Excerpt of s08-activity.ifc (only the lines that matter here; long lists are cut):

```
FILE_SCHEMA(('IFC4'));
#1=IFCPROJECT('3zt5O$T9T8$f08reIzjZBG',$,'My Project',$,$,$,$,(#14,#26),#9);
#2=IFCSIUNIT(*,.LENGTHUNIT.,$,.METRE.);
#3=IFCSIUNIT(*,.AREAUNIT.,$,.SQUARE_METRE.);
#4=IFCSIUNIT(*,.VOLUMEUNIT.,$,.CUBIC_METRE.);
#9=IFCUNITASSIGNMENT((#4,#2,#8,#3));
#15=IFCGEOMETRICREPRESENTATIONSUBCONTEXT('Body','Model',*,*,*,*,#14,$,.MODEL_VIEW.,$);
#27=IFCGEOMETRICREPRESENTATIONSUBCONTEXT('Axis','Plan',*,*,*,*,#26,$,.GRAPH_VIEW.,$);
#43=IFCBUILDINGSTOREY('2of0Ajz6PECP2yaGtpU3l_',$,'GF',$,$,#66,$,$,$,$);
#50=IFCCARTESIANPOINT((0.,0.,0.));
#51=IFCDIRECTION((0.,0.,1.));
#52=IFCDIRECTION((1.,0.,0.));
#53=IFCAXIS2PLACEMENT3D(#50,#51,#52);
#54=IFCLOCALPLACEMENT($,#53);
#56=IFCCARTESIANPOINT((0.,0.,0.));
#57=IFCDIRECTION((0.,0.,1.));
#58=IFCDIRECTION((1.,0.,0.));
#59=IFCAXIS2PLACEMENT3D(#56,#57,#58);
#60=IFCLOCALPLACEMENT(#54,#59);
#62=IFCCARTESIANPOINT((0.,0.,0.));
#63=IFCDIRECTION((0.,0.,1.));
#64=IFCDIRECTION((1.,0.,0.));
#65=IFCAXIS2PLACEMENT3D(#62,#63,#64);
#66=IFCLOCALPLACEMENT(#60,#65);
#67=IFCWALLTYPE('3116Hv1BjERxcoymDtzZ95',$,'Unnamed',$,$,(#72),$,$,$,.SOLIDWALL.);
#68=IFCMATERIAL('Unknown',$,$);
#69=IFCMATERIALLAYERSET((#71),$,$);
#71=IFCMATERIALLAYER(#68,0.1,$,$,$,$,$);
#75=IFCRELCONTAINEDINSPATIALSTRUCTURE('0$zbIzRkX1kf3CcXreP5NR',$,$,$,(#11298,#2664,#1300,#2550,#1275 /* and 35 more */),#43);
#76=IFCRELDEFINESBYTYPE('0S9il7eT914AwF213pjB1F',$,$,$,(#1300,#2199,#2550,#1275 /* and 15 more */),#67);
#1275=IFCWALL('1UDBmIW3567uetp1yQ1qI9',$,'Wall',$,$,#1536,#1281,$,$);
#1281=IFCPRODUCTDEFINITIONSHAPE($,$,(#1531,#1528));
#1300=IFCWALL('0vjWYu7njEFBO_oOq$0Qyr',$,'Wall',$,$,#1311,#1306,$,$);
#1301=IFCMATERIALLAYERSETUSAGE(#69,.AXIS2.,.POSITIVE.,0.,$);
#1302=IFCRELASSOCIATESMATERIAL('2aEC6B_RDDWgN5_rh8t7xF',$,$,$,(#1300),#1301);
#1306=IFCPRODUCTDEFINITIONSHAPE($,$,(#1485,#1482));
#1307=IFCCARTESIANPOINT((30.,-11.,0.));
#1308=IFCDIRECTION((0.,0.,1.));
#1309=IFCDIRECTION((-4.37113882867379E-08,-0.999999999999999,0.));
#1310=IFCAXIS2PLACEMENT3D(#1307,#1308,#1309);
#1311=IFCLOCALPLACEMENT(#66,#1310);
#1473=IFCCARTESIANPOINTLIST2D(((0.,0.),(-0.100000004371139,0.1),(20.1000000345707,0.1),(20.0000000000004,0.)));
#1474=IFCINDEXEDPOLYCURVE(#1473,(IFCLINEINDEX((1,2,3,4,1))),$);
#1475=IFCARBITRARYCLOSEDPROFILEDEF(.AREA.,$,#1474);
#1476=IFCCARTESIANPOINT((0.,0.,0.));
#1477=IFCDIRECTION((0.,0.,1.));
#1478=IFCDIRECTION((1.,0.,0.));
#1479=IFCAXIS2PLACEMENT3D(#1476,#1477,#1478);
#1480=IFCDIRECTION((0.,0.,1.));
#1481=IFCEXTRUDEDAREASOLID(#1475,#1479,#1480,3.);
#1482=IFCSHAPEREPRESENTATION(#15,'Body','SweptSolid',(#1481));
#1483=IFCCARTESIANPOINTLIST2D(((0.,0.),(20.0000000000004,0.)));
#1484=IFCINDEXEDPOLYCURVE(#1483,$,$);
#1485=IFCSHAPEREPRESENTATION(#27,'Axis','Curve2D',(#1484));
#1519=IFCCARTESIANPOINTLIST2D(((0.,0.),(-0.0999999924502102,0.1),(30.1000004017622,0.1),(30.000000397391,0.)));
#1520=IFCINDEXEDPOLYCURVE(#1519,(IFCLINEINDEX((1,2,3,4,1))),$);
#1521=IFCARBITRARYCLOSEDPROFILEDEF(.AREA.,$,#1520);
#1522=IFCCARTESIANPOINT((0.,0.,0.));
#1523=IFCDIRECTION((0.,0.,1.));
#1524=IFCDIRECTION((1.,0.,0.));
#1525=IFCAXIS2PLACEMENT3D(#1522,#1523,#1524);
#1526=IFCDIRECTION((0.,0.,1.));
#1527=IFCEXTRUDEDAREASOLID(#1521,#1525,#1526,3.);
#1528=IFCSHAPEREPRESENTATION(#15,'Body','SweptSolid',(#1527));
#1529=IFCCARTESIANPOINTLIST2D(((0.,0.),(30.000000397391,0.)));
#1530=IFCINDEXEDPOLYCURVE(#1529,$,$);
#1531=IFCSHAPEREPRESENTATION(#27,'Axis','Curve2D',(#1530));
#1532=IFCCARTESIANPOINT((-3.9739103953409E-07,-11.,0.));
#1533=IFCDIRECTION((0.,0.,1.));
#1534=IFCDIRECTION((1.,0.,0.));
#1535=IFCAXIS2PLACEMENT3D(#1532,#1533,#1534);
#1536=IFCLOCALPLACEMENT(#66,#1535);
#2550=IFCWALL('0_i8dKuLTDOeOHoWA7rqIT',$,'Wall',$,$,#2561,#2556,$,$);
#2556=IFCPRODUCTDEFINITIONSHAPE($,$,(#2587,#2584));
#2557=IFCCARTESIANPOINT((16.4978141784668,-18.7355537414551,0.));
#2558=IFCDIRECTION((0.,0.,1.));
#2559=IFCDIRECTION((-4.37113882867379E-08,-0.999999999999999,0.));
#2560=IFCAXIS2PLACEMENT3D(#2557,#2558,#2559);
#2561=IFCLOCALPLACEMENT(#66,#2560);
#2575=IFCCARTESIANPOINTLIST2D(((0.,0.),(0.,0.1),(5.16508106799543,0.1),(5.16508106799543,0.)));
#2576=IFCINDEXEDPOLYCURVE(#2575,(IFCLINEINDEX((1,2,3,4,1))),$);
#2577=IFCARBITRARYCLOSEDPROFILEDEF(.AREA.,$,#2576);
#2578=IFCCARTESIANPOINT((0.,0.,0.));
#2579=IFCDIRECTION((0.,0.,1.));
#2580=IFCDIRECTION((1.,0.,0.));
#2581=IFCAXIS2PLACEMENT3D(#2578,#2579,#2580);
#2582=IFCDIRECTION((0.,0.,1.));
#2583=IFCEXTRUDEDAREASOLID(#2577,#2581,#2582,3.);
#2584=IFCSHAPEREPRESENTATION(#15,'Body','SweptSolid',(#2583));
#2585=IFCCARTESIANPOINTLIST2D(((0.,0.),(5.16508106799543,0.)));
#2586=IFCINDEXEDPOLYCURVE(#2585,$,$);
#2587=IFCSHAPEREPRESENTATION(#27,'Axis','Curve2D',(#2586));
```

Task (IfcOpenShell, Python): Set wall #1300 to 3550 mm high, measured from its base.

```python
import ifcopenshell
import ifcopenshell.geom
import ifcopenshell.util.representation
import ifcopenshell.util.shape

model = ifcopenshell.open("s08-activity.ifc")
settings = ifcopenshell.geom.settings()


def volume(element):
    """Net volume in cubic metres, openings subtracted."""
    shape = ifcopenshell.geom.create_shape(settings, element)
    return ifcopenshell.util.shape.get_volume(shape.geometry)


wall = model.by_guid("0vjWYu7njEFBO_oOq$0Qyr")
before = volume(wall)

body = ifcopenshell.util.representation.get_representation(wall, "Model", "Body")
solid = body.Items[0]
old_height = solid.Depth
solid.Depth = 3.55
after = volume(wall)

print(f"height {old_height:g} -> {solid.Depth:g}, volume {before:.3f} -> {after:.3f} m3")

model.write("s08-activity_v2.ifc")
```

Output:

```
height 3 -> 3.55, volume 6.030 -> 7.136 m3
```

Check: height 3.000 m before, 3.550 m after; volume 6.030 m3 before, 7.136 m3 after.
